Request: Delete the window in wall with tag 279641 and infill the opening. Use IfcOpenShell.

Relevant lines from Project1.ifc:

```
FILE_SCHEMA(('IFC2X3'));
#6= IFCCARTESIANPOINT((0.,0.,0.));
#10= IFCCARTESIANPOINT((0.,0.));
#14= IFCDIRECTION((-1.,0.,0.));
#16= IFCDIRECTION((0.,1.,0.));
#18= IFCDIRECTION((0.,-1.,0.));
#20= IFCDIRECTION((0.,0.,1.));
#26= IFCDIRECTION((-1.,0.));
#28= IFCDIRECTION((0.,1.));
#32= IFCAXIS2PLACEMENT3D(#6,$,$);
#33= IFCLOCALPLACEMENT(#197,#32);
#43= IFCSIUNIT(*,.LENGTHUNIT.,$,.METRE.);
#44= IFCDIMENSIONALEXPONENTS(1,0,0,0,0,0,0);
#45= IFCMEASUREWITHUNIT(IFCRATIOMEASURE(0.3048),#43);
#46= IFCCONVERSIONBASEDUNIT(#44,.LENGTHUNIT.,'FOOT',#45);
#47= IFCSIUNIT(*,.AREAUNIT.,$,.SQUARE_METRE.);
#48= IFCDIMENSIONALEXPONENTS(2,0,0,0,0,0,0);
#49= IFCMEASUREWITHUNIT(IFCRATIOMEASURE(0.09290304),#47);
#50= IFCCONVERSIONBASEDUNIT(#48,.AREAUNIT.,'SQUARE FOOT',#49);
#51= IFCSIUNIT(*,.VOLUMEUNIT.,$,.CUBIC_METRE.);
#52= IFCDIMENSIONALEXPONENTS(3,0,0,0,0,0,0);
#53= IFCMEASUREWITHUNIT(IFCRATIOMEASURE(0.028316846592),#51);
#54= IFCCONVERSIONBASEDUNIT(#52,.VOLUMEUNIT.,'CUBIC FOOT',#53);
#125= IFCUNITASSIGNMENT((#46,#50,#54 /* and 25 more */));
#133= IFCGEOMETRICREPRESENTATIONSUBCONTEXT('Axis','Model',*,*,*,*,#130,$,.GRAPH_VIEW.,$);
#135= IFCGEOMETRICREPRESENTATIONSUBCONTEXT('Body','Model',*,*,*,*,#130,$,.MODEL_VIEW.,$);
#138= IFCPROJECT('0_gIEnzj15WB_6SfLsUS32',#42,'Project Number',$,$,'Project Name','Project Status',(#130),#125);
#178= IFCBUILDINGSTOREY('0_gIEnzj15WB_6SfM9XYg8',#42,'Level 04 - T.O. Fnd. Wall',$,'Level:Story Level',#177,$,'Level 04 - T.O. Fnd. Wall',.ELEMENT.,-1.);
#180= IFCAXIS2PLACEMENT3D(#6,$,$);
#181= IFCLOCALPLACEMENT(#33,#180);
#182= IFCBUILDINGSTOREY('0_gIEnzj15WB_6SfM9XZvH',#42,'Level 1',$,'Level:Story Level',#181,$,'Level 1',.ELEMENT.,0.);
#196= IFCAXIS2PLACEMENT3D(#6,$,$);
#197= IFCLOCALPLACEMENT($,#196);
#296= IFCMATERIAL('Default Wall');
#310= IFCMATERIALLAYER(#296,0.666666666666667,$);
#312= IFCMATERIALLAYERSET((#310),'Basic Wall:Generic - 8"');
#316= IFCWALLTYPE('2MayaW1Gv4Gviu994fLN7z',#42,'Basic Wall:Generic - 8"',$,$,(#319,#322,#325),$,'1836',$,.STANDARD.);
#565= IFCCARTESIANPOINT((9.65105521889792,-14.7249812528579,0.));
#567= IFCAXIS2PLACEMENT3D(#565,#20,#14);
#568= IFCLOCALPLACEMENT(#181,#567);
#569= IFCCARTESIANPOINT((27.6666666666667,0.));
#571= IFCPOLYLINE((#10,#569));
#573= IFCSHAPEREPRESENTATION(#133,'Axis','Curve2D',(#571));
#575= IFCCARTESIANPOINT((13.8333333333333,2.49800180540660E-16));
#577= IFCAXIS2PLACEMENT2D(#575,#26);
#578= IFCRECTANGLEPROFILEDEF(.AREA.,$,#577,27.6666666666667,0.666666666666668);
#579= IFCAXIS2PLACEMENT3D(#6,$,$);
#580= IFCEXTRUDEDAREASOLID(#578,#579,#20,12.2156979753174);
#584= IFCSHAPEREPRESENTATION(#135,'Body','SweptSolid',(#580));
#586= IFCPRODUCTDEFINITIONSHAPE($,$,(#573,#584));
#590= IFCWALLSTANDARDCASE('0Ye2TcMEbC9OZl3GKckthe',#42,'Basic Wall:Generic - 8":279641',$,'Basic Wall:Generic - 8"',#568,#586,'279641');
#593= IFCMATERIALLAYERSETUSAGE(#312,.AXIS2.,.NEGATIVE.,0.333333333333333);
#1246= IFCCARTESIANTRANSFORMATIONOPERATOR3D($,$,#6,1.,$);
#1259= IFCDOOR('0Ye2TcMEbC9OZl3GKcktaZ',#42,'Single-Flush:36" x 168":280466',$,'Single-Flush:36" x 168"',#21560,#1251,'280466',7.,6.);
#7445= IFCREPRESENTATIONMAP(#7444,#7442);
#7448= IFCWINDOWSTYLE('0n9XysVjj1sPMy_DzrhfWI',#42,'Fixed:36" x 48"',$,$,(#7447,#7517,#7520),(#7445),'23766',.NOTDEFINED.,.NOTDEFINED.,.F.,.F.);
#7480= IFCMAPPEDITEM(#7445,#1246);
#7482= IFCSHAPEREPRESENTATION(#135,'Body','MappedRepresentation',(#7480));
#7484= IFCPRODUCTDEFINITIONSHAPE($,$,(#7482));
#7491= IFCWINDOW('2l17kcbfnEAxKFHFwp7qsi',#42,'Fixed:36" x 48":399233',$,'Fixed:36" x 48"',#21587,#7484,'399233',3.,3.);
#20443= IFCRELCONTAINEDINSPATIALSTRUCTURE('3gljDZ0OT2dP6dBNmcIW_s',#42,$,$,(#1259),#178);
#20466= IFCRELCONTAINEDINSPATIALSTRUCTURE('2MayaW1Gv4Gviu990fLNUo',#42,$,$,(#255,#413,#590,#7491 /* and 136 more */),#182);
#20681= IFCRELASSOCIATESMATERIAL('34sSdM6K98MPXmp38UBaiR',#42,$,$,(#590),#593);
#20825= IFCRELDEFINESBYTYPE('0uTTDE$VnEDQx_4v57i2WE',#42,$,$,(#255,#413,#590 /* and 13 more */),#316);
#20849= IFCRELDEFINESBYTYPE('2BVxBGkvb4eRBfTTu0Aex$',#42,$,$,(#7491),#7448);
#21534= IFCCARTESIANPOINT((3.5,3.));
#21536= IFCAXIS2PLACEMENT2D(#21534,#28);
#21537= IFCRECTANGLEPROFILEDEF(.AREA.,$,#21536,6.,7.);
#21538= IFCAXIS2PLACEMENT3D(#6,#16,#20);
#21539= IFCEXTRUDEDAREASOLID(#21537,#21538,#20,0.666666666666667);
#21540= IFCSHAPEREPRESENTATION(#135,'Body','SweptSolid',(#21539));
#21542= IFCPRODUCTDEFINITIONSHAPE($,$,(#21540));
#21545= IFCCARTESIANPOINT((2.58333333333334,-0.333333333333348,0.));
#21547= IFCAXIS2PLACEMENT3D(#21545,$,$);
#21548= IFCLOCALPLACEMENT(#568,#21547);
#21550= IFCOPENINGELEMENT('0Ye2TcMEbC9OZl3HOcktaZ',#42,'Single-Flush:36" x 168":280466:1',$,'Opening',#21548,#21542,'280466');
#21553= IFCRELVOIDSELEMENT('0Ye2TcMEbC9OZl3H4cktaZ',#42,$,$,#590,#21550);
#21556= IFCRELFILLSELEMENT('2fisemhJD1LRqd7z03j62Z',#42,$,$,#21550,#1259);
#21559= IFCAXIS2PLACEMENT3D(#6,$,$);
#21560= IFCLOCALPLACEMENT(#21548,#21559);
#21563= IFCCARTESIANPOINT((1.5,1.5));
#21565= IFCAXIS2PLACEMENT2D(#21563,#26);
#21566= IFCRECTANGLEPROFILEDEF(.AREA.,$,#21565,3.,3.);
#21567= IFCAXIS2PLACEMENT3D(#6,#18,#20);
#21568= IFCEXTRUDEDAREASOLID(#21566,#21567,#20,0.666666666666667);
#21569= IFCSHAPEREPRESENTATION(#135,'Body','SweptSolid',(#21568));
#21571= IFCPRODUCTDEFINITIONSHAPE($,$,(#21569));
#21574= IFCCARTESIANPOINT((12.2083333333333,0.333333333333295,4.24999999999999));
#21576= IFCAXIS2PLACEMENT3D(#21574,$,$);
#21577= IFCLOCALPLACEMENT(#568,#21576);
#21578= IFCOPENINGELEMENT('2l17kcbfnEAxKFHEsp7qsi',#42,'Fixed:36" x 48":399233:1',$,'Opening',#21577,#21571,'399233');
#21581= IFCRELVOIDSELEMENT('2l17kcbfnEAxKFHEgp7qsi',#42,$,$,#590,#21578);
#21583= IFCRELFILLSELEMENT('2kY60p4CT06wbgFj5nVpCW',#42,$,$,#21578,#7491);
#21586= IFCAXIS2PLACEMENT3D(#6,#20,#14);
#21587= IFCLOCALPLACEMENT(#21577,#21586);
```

```python
import ifcopenshell
import ifcopenshell.api.feature
import ifcopenshell.api.root
import ifcopenshell.geom
import ifcopenshell.util.shape

model = ifcopenshell.open("Project1.ifc")
settings = ifcopenshell.geom.settings()


def volume(element):
    """Net volume in cubic metres, openings subtracted."""
    shape = ifcopenshell.geom.create_shape(settings, element)
    return ifcopenshell.util.shape.get_volume(shape.geometry)


window = model.by_id(7491)
opening = window.FillsVoids[0].RelatingOpeningElement
wall = opening.VoidsElements[0].RelatingBuildingElement
before = volume(wall)

ifcopenshell.api.root.remove_product(model, product=window)
ifcopenshell.api.feature.remove_feature(model, feature=opening)

after = volume(wall)

print(f"wall volume {before:.3f} -> {after:.3f} m3")

model.write("Project1_edited.ifc")
```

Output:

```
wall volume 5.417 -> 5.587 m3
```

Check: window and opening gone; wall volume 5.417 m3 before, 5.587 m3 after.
